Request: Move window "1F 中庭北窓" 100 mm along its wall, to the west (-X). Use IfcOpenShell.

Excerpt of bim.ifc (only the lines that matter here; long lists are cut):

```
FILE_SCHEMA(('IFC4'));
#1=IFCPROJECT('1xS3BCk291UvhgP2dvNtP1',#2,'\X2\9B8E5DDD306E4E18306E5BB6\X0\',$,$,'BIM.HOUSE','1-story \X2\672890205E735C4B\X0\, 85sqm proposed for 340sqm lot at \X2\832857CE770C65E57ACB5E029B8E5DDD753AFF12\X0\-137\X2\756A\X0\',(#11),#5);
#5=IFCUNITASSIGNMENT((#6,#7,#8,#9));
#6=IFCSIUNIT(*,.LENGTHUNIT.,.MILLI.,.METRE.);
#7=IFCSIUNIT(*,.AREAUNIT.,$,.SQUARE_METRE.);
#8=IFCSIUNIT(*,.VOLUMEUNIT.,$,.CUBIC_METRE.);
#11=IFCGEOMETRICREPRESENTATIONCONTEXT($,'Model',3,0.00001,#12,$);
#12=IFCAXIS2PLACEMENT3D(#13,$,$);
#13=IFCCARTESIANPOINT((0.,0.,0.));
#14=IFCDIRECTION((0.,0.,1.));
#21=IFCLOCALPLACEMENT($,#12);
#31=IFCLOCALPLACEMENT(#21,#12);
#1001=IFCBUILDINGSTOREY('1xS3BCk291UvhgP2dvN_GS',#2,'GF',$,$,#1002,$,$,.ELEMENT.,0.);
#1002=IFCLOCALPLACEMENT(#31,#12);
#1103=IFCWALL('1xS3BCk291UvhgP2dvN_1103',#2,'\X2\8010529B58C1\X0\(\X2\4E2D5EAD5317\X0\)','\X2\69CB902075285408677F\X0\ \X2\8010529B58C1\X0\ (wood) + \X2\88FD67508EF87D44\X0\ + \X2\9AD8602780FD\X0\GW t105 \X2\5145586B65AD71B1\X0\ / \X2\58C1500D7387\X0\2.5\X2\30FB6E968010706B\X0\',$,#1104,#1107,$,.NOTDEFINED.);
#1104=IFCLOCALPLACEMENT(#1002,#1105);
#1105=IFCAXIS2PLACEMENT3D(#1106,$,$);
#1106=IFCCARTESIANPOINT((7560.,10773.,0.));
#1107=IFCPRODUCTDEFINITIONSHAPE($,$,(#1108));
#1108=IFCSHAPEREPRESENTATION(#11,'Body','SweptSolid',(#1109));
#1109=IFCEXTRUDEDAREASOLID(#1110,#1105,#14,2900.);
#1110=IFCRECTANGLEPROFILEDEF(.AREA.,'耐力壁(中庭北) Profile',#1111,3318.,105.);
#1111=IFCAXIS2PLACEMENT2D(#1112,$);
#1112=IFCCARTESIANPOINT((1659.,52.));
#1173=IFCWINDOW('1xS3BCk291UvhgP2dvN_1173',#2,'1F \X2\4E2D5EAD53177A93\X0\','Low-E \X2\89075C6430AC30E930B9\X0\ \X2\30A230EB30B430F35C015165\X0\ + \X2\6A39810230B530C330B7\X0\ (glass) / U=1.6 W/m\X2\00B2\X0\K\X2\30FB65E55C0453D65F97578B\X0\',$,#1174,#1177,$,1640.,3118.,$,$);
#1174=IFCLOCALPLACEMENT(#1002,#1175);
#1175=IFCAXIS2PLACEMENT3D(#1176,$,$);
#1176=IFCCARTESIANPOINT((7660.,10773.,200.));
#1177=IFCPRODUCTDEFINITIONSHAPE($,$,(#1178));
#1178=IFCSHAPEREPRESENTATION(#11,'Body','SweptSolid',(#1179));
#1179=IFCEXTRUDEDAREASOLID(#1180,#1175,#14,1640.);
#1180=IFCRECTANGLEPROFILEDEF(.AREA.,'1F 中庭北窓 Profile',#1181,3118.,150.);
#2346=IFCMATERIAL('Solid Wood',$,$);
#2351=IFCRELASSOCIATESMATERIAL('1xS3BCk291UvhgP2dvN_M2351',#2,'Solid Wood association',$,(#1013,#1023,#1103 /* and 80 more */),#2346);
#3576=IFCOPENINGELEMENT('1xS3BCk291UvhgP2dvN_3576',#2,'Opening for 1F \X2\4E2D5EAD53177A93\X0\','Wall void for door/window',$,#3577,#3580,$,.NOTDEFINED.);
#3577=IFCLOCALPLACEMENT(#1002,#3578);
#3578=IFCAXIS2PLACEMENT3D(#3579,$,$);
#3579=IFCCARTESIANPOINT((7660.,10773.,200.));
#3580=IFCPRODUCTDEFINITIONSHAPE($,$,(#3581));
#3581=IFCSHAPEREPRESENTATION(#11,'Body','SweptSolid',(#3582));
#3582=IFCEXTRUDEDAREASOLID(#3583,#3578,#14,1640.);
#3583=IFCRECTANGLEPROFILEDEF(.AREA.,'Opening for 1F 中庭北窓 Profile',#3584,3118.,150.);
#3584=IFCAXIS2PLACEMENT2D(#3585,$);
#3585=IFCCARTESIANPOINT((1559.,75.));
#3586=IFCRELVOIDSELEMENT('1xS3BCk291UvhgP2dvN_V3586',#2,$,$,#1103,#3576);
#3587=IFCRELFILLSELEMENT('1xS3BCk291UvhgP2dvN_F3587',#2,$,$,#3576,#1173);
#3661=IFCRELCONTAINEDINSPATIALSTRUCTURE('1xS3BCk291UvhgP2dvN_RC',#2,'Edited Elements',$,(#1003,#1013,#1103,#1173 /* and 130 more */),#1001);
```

```python
import ifcopenshell
import ifcopenshell.api.geometry
import ifcopenshell.util.placement
import ifcopenshell.util.unit

model = ifcopenshell.open("bim.ifc")
unit_scale = ifcopenshell.util.unit.calculate_unit_scale(model)

window = model.by_guid("1xS3BCk291UvhgP2dvN_1173")
opening = window.FillsVoids[0].RelatingOpeningElement
wall = opening.VoidsElements[0].RelatingBuildingElement

wall_matrix = ifcopenshell.util.placement.get_local_placement(wall.ObjectPlacement)
shift = wall_matrix[:3, 0] * -0.1 / unit_scale
before = ifcopenshell.util.placement.get_local_placement(window.ObjectPlacement)[:3, 3].copy()

# The window is not placed relative to its opening, so move both.
for product in (opening, window):
    matrix = ifcopenshell.util.placement.get_local_placement(product.ObjectPlacement)
    matrix[:3, 3] += shift
    ifcopenshell.api.geometry.edit_object_placement(model, product=product, matrix=matrix, is_si=False)

after = ifcopenshell.util.placement.get_local_placement(window.ObjectPlacement)[:3, 3]
print("window moved by", (after - before).round(3) + 0.0)

model.write("bim_v2.ifc")
```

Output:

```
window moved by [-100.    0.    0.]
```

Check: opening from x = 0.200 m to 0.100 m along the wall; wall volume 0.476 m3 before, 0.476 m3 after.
